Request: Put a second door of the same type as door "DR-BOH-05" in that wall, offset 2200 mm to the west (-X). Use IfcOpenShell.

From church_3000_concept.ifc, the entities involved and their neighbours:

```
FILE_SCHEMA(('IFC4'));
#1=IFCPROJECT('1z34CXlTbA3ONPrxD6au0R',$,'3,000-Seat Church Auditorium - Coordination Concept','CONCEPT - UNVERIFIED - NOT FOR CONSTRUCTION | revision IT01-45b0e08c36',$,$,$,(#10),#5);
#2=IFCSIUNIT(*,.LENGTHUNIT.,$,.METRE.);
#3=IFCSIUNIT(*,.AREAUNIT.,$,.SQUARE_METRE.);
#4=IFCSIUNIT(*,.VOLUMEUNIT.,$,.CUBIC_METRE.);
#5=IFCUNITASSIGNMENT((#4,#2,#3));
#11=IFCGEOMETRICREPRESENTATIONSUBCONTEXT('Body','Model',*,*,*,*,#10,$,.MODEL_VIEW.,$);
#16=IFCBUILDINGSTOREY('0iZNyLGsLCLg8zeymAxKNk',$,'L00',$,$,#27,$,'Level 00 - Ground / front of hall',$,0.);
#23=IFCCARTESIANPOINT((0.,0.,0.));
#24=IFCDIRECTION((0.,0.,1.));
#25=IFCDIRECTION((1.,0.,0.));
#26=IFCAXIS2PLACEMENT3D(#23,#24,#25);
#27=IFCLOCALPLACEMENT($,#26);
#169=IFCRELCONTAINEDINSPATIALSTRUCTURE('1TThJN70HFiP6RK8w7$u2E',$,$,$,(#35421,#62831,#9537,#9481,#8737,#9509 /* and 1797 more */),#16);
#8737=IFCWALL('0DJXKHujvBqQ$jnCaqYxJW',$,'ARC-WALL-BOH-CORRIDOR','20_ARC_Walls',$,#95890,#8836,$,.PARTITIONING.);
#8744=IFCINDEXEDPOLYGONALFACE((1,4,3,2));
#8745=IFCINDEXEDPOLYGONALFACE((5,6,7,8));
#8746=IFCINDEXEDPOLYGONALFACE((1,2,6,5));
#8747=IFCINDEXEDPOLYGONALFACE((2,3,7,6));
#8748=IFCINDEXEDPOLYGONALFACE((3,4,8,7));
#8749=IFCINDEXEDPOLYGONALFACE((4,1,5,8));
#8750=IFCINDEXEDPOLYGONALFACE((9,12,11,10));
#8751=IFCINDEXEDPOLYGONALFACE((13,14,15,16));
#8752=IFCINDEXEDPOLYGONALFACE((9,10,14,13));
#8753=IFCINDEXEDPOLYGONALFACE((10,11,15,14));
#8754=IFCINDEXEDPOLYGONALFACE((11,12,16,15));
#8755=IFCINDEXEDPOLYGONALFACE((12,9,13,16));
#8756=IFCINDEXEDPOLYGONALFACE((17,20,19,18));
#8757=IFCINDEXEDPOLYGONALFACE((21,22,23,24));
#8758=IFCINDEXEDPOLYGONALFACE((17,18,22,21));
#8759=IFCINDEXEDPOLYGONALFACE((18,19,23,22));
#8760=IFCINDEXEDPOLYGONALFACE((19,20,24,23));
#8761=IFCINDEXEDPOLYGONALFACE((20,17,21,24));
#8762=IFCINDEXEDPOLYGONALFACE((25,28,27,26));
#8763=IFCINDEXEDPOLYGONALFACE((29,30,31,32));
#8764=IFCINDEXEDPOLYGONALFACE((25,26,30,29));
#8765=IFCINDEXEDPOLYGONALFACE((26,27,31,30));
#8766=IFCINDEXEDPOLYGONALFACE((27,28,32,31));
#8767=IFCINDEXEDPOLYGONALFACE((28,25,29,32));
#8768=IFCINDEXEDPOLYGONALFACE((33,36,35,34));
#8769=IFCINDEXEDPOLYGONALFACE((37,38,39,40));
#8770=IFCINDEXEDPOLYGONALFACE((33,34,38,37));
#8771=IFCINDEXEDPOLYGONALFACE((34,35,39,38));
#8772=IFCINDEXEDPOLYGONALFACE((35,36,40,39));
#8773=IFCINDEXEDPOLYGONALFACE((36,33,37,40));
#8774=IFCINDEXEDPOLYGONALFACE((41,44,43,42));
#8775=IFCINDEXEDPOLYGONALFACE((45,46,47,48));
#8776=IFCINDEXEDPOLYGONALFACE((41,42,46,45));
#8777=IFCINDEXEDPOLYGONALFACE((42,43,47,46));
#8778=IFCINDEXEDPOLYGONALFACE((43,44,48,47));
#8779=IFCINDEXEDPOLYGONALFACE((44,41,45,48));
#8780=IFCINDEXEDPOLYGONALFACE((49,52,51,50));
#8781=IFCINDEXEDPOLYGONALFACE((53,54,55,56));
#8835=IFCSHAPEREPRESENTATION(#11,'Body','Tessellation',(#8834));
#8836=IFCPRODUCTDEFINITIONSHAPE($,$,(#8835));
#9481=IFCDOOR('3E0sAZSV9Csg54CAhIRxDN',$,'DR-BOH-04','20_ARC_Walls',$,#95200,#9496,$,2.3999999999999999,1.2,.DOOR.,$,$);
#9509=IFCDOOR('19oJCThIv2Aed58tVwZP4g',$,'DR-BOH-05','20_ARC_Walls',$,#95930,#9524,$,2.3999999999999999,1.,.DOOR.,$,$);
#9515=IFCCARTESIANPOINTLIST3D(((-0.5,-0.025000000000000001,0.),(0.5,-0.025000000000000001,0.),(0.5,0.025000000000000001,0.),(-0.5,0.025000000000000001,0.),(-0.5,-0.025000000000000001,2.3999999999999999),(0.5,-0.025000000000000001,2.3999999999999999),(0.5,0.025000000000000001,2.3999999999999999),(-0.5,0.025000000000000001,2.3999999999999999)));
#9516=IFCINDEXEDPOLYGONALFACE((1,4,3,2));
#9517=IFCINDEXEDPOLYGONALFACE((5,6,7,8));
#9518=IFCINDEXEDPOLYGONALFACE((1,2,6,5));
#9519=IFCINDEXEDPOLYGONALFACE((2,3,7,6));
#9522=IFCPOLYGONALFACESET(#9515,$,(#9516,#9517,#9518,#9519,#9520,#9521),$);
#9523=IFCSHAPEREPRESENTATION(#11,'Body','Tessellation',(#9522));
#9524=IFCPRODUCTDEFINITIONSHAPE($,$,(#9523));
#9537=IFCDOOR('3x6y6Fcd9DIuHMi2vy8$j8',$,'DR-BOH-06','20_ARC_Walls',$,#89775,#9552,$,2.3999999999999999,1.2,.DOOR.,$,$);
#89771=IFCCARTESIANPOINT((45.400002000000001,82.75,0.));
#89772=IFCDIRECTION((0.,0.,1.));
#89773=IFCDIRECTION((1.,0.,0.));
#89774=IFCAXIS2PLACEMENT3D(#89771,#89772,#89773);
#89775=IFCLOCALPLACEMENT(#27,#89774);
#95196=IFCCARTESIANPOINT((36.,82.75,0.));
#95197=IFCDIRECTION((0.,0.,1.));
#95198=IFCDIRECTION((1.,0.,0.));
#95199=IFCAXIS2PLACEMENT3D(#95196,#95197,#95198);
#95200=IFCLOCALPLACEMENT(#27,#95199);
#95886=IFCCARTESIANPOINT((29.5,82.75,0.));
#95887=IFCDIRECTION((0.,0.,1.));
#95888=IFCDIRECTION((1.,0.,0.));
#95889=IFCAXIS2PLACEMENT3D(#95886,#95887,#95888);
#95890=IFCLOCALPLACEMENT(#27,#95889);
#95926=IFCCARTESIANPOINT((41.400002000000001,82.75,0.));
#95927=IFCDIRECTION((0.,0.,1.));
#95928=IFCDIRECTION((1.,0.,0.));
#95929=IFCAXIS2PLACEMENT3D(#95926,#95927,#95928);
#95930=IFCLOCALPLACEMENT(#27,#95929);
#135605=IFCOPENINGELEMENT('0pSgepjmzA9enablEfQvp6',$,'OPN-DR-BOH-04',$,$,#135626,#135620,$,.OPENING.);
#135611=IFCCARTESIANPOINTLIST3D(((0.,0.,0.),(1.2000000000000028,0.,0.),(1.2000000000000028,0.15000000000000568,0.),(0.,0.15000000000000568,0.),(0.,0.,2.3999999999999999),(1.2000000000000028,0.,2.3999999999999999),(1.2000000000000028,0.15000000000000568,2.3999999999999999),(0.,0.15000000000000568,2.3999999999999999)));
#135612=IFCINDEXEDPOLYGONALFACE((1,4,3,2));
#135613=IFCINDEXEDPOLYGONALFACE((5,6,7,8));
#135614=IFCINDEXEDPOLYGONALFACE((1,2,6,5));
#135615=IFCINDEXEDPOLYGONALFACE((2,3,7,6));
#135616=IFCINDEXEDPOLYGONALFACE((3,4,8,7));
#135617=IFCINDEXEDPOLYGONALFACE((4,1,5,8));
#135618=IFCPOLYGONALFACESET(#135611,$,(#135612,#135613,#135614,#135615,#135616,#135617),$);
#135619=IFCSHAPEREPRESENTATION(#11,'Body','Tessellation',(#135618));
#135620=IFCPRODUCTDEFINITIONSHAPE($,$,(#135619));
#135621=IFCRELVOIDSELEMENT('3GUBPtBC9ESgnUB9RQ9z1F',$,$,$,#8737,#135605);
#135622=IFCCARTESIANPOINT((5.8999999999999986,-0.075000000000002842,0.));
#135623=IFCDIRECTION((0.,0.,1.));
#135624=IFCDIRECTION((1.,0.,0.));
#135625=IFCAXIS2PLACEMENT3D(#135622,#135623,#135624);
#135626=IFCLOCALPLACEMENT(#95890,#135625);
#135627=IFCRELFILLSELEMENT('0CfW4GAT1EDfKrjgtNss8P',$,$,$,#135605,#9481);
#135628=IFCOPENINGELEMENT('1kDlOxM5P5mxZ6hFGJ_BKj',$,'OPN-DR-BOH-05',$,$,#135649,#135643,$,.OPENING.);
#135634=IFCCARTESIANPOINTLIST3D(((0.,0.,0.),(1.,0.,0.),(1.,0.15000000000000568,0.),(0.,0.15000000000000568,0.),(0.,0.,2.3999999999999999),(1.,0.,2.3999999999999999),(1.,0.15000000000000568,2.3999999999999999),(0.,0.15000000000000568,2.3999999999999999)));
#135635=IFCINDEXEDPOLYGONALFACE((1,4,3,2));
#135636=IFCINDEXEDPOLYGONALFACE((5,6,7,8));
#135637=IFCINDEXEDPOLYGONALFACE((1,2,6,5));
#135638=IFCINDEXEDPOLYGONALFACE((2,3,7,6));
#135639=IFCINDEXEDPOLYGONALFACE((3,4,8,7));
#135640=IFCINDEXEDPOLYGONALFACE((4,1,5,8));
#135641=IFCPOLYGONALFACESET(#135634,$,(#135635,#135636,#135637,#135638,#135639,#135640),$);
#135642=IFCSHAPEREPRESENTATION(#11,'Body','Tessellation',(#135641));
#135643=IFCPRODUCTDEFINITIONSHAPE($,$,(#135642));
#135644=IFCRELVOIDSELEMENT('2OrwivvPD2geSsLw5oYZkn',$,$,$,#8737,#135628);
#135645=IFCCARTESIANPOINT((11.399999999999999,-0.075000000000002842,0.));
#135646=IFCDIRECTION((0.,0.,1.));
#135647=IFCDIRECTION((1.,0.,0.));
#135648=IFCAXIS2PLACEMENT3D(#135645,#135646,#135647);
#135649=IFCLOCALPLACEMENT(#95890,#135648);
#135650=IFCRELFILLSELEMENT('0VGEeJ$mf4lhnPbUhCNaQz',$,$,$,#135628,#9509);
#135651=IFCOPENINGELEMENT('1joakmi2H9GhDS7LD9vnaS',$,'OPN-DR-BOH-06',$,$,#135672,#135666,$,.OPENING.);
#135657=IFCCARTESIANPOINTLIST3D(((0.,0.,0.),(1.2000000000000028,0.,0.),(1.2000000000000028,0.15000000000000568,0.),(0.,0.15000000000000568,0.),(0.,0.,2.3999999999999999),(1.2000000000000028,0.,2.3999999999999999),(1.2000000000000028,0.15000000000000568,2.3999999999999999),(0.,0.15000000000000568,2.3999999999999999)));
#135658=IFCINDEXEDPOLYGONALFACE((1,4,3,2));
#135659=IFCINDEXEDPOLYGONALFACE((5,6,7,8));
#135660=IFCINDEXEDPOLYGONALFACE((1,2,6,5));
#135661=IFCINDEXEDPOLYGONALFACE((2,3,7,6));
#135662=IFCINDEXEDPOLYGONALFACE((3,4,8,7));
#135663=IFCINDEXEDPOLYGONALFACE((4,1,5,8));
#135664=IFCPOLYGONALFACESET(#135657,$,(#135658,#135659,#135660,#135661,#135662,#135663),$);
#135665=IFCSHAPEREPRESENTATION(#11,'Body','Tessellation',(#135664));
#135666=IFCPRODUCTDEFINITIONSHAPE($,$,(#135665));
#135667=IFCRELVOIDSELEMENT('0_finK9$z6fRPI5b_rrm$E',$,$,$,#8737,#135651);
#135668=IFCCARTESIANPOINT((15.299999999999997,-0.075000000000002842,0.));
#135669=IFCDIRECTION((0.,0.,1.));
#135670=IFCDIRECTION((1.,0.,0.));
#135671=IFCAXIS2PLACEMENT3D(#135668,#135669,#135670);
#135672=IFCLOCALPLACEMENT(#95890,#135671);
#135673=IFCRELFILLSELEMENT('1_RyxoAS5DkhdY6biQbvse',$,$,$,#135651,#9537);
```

```python
import ifcopenshell
import ifcopenshell.api.feature
import ifcopenshell.api.geometry
import ifcopenshell.api.root
import ifcopenshell.geom
import ifcopenshell.util.element
import ifcopenshell.util.placement
import ifcopenshell.util.shape

model = ifcopenshell.open("church_3000_concept.ifc")
settings = ifcopenshell.geom.settings()


def volume(element):
    """Net volume in cubic metres, openings subtracted."""
    shape = ifcopenshell.geom.create_shape(settings, element)
    return ifcopenshell.util.shape.get_volume(shape.geometry)


door = model.by_guid("19oJCThIv2Aed58tVwZP4g")
opening = door.FillsVoids[0].RelatingOpeningElement
wall = opening.VoidsElements[0].RelatingBuildingElement
before = volume(wall)
shift = ifcopenshell.util.placement.get_local_placement(wall.ObjectPlacement)[:3, 0] * -2.2

# copy_class copies the void relationship, type, container and properties, but no geometry.
new_opening = ifcopenshell.api.root.copy_class(model, product=opening)
new_opening.Representation = ifcopenshell.util.element.copy_deep(
    model, opening.Representation, exclude=["IfcGeometricRepresentationContext", "IfcRepresentationMap"]
)
new_door = ifcopenshell.api.root.copy_class(model, product=door)
new_door.Representation = ifcopenshell.util.element.copy_deep(
    model, door.Representation, exclude=["IfcGeometricRepresentationContext", "IfcRepresentationMap"]
)
ifcopenshell.api.feature.add_filling(model, opening=new_opening, element=new_door)

for old, new in ((opening, new_opening), (door, new_door)):
    matrix = ifcopenshell.util.placement.get_local_placement(old.ObjectPlacement)
    matrix[:3, 3] += shift
    ifcopenshell.api.geometry.edit_object_placement(model, product=new, matrix=matrix, is_si=False)

after = volume(wall)

print(f"wall volume {before:.3f} -> {after:.3f} m3")

model.write("church_3000_concept_updated.ifc")
```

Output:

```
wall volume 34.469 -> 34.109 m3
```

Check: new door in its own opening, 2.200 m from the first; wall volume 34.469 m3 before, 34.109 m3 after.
